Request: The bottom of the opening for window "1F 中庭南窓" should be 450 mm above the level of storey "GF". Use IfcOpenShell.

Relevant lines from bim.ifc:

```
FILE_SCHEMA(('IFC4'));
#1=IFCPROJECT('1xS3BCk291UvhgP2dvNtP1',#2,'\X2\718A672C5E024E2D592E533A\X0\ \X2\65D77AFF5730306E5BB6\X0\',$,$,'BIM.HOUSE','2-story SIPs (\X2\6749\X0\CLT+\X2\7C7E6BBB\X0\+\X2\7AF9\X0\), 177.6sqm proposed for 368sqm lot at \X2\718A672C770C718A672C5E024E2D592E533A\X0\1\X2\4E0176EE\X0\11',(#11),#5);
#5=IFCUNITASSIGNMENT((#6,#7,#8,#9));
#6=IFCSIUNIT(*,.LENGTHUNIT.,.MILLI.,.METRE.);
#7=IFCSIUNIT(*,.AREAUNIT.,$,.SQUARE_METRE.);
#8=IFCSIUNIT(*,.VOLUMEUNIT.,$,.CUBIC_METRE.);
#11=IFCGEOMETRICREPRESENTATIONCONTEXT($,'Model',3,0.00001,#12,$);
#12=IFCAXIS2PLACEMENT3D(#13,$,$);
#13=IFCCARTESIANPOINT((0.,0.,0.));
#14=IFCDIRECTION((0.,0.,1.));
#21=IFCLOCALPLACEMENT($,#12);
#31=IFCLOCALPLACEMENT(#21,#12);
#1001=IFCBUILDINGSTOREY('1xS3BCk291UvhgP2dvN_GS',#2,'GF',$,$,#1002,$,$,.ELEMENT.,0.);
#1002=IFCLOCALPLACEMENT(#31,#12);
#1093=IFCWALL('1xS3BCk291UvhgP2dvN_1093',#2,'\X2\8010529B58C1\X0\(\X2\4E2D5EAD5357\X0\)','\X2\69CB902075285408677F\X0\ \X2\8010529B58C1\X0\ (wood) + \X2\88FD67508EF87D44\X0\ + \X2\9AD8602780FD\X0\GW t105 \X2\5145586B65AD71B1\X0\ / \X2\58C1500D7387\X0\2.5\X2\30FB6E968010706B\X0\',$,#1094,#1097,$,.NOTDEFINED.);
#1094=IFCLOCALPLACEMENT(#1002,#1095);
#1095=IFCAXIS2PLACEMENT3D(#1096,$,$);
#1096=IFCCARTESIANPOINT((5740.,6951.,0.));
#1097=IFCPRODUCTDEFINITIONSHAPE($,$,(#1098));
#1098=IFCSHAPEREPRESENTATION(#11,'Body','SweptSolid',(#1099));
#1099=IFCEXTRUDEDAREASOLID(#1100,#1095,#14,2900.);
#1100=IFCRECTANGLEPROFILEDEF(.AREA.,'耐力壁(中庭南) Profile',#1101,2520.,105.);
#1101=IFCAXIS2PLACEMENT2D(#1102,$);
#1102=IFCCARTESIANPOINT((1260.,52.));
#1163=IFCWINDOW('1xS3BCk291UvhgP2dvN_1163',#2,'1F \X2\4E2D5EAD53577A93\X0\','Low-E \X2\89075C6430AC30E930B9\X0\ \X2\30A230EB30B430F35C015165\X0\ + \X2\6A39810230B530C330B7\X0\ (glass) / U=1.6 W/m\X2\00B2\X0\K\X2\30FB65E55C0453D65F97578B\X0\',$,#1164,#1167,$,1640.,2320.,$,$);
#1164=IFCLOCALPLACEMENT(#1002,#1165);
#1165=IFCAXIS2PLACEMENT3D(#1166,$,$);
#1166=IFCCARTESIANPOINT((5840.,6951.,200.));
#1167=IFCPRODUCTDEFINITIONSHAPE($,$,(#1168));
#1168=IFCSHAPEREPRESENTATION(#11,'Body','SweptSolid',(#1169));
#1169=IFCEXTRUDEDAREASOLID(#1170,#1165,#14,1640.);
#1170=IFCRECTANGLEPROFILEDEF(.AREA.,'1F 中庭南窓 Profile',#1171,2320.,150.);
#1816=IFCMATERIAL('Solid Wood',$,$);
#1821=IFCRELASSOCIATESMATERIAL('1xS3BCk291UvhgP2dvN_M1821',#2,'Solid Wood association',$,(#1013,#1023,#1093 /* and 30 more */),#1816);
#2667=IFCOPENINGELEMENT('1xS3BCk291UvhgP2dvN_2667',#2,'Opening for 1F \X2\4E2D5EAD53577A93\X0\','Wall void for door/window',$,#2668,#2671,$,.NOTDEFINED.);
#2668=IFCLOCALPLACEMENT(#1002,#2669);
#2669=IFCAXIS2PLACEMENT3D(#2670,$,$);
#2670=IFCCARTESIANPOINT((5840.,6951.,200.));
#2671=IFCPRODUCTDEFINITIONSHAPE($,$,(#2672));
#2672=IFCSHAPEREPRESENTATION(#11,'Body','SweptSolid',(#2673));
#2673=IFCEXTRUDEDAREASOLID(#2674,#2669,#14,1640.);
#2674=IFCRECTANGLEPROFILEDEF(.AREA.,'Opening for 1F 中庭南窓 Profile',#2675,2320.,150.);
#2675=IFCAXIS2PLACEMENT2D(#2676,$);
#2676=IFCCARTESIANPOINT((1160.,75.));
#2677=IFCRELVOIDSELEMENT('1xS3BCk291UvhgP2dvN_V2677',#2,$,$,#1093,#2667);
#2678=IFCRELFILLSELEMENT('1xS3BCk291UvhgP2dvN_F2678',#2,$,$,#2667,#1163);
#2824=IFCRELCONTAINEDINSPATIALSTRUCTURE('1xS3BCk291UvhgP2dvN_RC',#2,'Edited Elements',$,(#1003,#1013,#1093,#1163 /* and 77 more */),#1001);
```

```python
import numpy as np
import ifcopenshell
import ifcopenshell.api.geometry
import ifcopenshell.geom
import ifcopenshell.util.element
import ifcopenshell.util.placement
import ifcopenshell.util.shape
import ifcopenshell.util.unit

model = ifcopenshell.open("bim.ifc")
unit_scale = ifcopenshell.util.unit.calculate_unit_scale(model)

window = model.by_guid("1xS3BCk291UvhgP2dvN_1163")
opening = window.FillsVoids[0].RelatingOpeningElement
storey = ifcopenshell.util.element.get_container(window, ifc_class="IfcBuildingStorey")
level = ifcopenshell.util.placement.get_local_placement(storey.ObjectPlacement)[2, 3]

# The opening's origin need not be at the sill, so measure its lowest point.
shape = ifcopenshell.geom.create_shape(ifcopenshell.geom.settings(), opening)
bottom = ifcopenshell.util.shape.get_shape_bottom_elevation(shape, shape.geometry) / unit_scale
dz = level + 0.45 / unit_scale - bottom

shift = np.array([0.0, 0.0, dz])
# The window is not placed relative to its opening, so move both.
for product in (opening, window):
    matrix = ifcopenshell.util.placement.get_local_placement(product.ObjectPlacement)
    matrix[:3, 3] += shift
    ifcopenshell.api.geometry.edit_object_placement(model, product=product, matrix=matrix, is_si=False)

print(f"moved by {dz * unit_scale:+.3f} m")

model.write("bim_rev.ifc")
```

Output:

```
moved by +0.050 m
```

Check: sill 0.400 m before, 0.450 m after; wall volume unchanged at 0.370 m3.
